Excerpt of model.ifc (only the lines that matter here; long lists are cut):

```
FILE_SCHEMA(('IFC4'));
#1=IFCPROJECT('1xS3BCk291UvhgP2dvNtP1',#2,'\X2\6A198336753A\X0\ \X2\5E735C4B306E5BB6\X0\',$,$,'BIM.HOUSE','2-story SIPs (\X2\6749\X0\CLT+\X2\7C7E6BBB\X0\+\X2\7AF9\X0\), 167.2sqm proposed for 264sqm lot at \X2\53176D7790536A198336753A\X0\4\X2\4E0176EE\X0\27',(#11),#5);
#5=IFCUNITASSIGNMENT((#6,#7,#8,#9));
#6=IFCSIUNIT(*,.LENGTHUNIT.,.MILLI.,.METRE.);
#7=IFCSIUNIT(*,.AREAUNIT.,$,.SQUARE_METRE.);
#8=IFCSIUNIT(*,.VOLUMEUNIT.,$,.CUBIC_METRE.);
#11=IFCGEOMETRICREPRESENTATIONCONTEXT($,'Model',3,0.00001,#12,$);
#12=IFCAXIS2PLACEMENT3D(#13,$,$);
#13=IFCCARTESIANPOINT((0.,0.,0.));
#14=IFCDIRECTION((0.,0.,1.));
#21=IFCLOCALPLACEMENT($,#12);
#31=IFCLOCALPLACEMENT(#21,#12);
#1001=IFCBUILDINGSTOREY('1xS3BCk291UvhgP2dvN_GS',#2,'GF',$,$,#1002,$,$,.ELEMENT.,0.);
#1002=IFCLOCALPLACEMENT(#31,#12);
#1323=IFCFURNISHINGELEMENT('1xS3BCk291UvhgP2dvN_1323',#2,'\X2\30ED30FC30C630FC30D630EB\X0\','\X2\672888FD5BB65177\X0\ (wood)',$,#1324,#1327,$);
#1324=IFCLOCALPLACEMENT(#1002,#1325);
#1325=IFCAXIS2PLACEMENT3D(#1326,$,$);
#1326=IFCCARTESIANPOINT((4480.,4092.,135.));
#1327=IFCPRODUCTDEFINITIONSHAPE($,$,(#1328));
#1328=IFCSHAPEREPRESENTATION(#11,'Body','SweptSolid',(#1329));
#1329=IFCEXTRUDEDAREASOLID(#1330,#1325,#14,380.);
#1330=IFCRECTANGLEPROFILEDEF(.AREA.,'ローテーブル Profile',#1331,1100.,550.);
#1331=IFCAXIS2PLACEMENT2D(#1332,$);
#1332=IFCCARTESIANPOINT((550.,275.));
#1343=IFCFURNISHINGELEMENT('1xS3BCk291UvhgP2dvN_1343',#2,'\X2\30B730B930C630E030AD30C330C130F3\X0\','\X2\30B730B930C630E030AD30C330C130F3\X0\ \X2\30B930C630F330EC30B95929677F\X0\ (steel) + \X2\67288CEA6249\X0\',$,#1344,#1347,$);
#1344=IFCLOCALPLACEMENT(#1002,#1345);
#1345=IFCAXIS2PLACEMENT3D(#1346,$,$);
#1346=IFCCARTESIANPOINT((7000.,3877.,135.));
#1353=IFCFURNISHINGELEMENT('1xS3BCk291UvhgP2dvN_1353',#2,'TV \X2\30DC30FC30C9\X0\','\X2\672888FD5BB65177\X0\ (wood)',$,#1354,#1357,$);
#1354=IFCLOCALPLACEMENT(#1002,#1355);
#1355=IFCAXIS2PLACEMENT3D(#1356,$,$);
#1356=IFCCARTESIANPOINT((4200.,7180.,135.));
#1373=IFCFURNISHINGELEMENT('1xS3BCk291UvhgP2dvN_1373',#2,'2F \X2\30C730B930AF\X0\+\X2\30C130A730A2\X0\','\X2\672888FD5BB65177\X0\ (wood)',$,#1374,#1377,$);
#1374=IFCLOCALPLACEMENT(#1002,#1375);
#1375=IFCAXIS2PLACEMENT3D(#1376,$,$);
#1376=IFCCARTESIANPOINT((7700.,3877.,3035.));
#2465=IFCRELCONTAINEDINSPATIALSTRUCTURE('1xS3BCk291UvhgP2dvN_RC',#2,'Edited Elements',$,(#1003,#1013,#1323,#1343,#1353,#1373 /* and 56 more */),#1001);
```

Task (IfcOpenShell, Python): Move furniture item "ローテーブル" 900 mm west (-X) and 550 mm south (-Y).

```python
import ifcopenshell
import ifcopenshell.api.geometry
import ifcopenshell.util.placement

model = ifcopenshell.open("model.ifc")

item = model.by_id(1323)
matrix = ifcopenshell.util.placement.get_local_placement(item.ObjectPlacement)
matrix[0, 3] -= 900.0
matrix[1, 3] -= 550.0
ifcopenshell.api.geometry.edit_object_placement(model, product=item, matrix=matrix, is_si=False)

print(ifcopenshell.util.placement.get_local_placement(item.ObjectPlacement).round(3) + 0.0)

model.write("model_rev.ifc")
```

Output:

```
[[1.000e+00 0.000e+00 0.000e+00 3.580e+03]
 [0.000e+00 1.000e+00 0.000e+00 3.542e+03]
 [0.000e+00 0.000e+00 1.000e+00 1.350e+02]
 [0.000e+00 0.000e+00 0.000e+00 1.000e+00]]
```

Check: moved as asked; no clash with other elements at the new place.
